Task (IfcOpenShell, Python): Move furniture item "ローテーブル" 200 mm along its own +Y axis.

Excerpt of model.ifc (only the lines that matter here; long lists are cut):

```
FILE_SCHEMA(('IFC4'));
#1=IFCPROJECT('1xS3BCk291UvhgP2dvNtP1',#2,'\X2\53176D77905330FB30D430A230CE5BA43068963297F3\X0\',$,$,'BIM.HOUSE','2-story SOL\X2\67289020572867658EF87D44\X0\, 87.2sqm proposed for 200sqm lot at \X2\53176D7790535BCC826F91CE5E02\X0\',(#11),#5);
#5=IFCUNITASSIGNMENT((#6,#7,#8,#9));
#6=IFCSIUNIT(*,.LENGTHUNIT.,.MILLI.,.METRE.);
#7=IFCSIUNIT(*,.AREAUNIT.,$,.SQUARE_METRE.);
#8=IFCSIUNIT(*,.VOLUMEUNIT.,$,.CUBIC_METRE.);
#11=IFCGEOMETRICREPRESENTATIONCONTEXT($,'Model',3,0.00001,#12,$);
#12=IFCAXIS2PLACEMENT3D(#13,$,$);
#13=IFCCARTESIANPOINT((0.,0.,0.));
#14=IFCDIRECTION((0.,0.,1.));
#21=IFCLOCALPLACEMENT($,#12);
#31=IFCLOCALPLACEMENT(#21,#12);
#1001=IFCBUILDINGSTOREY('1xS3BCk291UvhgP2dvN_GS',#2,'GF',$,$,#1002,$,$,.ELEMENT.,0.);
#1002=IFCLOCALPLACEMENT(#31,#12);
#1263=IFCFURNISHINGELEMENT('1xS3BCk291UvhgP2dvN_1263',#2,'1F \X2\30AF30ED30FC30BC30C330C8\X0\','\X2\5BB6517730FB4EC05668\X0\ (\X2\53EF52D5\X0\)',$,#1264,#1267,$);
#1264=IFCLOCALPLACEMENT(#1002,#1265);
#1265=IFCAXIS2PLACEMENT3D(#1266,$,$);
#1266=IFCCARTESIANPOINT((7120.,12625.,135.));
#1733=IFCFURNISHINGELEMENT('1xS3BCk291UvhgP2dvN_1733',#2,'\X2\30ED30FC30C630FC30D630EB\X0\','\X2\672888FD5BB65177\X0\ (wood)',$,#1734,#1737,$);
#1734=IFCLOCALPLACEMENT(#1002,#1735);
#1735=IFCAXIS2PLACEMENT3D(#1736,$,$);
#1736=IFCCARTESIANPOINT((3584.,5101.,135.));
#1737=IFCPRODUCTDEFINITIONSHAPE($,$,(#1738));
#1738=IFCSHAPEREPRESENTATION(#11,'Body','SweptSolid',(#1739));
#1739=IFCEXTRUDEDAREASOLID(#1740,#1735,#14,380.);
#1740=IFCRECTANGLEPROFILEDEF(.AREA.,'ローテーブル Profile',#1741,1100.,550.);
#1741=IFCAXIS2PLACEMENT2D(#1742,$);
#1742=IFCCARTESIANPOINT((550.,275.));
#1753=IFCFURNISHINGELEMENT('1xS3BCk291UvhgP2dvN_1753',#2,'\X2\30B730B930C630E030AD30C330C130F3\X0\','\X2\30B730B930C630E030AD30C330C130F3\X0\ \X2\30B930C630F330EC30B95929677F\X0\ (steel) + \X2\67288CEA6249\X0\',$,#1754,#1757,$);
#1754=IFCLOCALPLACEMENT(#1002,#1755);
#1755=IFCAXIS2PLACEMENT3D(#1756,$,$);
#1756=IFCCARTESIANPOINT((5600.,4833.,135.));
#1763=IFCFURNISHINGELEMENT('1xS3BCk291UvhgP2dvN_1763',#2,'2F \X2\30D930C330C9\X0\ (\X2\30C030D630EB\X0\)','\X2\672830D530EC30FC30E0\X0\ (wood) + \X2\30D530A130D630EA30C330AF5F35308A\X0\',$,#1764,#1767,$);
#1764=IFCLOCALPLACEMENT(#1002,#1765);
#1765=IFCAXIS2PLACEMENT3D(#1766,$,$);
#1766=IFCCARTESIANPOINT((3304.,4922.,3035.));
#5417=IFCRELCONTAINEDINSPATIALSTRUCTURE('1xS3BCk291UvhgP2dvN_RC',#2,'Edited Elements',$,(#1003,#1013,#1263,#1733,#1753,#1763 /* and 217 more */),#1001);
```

```python
import ifcopenshell
import ifcopenshell.api.geometry
import ifcopenshell.util.placement
import ifcopenshell.util.unit

model = ifcopenshell.open("model.ifc")
unit_scale = ifcopenshell.util.unit.calculate_unit_scale(model)

item = model.by_guid("1xS3BCk291UvhgP2dvN_1733")
matrix = ifcopenshell.util.placement.get_local_placement(item.ObjectPlacement)
matrix[:3, 3] += matrix[:3, 1] * 0.2 / unit_scale
ifcopenshell.api.geometry.edit_object_placement(model, product=item, matrix=matrix, is_si=False)

print(ifcopenshell.util.placement.get_local_placement(item.ObjectPlacement).round(3) + 0.0)

model.write("model_rev.ifc")
```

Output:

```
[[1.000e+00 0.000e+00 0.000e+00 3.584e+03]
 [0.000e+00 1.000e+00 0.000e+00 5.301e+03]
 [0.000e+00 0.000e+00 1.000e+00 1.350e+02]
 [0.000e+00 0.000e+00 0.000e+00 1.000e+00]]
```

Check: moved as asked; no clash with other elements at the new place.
